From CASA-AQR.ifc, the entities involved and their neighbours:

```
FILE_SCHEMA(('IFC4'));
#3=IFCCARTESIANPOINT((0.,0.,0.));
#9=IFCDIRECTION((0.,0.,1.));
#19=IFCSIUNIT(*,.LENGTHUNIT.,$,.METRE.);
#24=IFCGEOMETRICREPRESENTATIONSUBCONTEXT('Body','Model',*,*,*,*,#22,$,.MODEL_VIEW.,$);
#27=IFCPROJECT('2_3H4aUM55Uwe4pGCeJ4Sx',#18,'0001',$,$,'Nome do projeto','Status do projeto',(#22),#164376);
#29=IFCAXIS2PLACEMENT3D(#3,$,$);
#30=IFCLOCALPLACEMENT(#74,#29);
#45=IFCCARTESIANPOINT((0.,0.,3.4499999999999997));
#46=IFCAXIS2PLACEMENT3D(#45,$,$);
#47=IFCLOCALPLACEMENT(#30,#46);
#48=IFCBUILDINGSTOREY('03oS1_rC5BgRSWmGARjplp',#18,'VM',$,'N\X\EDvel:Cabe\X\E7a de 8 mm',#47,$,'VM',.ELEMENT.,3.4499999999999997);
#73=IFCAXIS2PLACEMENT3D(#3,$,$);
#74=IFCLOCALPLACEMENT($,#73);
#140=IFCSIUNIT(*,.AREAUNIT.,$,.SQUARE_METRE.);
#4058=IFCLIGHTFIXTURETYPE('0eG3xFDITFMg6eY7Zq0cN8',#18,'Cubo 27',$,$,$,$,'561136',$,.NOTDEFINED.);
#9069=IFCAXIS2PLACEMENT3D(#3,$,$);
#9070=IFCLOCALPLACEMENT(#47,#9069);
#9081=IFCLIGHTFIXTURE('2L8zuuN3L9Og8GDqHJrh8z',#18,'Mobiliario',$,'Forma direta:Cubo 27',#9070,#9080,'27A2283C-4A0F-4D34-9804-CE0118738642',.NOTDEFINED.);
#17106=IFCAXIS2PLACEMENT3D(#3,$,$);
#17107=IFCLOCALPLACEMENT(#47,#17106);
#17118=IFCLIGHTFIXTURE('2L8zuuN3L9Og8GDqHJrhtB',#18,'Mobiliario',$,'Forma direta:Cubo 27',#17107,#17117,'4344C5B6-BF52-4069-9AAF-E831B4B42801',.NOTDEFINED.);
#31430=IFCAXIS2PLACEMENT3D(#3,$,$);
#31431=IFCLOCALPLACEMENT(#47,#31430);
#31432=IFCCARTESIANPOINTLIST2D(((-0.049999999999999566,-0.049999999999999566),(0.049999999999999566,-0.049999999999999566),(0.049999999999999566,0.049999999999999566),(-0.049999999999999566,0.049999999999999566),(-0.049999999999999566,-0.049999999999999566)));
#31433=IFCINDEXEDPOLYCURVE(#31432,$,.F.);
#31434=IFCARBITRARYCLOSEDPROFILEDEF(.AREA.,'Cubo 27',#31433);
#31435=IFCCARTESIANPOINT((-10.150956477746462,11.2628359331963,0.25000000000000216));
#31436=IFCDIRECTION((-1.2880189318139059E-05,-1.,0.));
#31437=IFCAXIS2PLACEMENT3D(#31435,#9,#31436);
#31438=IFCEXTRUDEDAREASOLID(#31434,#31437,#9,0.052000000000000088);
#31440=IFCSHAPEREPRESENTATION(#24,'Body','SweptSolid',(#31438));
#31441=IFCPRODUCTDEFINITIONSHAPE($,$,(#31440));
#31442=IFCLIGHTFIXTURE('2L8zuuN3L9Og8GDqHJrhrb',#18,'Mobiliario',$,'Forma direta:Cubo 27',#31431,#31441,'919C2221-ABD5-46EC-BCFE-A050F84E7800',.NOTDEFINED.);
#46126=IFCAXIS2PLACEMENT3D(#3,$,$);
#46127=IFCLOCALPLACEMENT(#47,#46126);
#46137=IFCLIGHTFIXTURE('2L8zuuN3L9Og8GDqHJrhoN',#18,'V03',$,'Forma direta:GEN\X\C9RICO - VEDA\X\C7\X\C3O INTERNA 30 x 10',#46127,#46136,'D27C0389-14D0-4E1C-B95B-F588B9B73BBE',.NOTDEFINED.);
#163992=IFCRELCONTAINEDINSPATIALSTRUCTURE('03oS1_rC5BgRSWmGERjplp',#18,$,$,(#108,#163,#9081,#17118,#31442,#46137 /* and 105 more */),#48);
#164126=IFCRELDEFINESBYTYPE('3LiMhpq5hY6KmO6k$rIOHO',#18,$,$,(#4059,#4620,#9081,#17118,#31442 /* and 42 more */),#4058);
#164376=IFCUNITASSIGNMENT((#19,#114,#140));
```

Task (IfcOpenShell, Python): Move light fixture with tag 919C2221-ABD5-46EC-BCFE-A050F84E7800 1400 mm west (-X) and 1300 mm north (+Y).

```python
import ifcopenshell
import ifcopenshell.api.geometry
import ifcopenshell.util.placement
import ifcopenshell.util.unit

model = ifcopenshell.open("CASA-AQR.ifc")
unit_scale = ifcopenshell.util.unit.calculate_unit_scale(model)

item = model.by_id(31442)
matrix = ifcopenshell.util.placement.get_local_placement(item.ObjectPlacement)
matrix[0, 3] -= 1.4 / unit_scale
matrix[1, 3] += 1.3 / unit_scale
ifcopenshell.api.geometry.edit_object_placement(model, product=item, matrix=matrix, is_si=False)

print(ifcopenshell.util.placement.get_local_placement(item.ObjectPlacement).round(3) + 0.0)

model.write("CASA-AQR_v2.ifc")
```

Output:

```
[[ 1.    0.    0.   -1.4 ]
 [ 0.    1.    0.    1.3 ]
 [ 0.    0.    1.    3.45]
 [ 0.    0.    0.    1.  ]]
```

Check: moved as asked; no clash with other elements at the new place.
